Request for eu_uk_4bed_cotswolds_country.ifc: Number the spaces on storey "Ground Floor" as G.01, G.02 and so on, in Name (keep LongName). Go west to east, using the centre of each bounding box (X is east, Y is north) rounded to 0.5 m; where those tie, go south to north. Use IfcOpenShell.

First a look at what the model holds.

```python
import ifcopenshell
import ifcopenshell.util.element
import ifcopenshell.util.placement

model = ifcopenshell.open("eu_uk_4bed_cotswolds_country.ifc")
print(model.schema)
storey = next(s for s in model.by_type("IfcBuildingStorey") if s.Name == "Ground Floor")
spaces = [e for e in ifcopenshell.util.element.get_decomposition(storey) if e.is_a("IfcSpace")]
for e in sorted(spaces, key=lambda e: e.id()):
    origin = ifcopenshell.util.placement.get_local_placement(e.ObjectPlacement)[:3, 3]
    print(e.id(), e.Name, e.LongName, origin.round(2) + 0.0, sep=" | ")
```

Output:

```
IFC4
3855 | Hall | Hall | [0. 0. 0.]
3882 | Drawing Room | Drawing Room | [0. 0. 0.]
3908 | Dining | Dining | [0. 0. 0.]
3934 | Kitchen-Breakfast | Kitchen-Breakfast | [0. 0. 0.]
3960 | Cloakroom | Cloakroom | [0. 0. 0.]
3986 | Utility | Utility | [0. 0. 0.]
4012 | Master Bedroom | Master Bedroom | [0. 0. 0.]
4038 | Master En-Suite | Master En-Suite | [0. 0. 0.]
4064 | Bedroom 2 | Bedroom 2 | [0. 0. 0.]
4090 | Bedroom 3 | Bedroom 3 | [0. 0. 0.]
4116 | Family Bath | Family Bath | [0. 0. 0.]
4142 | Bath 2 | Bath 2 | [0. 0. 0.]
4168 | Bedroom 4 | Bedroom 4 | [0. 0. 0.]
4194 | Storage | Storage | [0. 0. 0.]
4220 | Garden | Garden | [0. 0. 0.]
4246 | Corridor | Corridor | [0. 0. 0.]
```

```python
import ifcopenshell
import ifcopenshell.geom
import ifcopenshell.util.element
import ifcopenshell.util.shape

model = ifcopenshell.open("eu_uk_4bed_cotswolds_country.ifc")
settings = ifcopenshell.geom.settings()
settings.set("use-world-coords", True)


def centre(element):
    shape = ifcopenshell.geom.create_shape(settings, element)
    return ifcopenshell.util.shape.get_bbox_centroid(shape.geometry)


storey = next(s for s in model.by_type("IfcBuildingStorey") if s.Name == "Ground Floor")
spaces = [e for e in ifcopenshell.util.element.get_decomposition(storey) if e.is_a("IfcSpace")]

# Insertion points can sit at a corner or the storey origin, so sort by the geometry (in metres).
centres = {e: centre(e) for e in spaces}
spaces.sort(key=lambda e: (round(centres[e][0] / 0.5), centres[e][1]))

for i, e in enumerate(spaces, start=1):
    number = f"G.{i:02d}"
    e.Name = number
    print(e.id(), number)

model.write("eu_uk_4bed_cotswolds_country_updated.ifc")
```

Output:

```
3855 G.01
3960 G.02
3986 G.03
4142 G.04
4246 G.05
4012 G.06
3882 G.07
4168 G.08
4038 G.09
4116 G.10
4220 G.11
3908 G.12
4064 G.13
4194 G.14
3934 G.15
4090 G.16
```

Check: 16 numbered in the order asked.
